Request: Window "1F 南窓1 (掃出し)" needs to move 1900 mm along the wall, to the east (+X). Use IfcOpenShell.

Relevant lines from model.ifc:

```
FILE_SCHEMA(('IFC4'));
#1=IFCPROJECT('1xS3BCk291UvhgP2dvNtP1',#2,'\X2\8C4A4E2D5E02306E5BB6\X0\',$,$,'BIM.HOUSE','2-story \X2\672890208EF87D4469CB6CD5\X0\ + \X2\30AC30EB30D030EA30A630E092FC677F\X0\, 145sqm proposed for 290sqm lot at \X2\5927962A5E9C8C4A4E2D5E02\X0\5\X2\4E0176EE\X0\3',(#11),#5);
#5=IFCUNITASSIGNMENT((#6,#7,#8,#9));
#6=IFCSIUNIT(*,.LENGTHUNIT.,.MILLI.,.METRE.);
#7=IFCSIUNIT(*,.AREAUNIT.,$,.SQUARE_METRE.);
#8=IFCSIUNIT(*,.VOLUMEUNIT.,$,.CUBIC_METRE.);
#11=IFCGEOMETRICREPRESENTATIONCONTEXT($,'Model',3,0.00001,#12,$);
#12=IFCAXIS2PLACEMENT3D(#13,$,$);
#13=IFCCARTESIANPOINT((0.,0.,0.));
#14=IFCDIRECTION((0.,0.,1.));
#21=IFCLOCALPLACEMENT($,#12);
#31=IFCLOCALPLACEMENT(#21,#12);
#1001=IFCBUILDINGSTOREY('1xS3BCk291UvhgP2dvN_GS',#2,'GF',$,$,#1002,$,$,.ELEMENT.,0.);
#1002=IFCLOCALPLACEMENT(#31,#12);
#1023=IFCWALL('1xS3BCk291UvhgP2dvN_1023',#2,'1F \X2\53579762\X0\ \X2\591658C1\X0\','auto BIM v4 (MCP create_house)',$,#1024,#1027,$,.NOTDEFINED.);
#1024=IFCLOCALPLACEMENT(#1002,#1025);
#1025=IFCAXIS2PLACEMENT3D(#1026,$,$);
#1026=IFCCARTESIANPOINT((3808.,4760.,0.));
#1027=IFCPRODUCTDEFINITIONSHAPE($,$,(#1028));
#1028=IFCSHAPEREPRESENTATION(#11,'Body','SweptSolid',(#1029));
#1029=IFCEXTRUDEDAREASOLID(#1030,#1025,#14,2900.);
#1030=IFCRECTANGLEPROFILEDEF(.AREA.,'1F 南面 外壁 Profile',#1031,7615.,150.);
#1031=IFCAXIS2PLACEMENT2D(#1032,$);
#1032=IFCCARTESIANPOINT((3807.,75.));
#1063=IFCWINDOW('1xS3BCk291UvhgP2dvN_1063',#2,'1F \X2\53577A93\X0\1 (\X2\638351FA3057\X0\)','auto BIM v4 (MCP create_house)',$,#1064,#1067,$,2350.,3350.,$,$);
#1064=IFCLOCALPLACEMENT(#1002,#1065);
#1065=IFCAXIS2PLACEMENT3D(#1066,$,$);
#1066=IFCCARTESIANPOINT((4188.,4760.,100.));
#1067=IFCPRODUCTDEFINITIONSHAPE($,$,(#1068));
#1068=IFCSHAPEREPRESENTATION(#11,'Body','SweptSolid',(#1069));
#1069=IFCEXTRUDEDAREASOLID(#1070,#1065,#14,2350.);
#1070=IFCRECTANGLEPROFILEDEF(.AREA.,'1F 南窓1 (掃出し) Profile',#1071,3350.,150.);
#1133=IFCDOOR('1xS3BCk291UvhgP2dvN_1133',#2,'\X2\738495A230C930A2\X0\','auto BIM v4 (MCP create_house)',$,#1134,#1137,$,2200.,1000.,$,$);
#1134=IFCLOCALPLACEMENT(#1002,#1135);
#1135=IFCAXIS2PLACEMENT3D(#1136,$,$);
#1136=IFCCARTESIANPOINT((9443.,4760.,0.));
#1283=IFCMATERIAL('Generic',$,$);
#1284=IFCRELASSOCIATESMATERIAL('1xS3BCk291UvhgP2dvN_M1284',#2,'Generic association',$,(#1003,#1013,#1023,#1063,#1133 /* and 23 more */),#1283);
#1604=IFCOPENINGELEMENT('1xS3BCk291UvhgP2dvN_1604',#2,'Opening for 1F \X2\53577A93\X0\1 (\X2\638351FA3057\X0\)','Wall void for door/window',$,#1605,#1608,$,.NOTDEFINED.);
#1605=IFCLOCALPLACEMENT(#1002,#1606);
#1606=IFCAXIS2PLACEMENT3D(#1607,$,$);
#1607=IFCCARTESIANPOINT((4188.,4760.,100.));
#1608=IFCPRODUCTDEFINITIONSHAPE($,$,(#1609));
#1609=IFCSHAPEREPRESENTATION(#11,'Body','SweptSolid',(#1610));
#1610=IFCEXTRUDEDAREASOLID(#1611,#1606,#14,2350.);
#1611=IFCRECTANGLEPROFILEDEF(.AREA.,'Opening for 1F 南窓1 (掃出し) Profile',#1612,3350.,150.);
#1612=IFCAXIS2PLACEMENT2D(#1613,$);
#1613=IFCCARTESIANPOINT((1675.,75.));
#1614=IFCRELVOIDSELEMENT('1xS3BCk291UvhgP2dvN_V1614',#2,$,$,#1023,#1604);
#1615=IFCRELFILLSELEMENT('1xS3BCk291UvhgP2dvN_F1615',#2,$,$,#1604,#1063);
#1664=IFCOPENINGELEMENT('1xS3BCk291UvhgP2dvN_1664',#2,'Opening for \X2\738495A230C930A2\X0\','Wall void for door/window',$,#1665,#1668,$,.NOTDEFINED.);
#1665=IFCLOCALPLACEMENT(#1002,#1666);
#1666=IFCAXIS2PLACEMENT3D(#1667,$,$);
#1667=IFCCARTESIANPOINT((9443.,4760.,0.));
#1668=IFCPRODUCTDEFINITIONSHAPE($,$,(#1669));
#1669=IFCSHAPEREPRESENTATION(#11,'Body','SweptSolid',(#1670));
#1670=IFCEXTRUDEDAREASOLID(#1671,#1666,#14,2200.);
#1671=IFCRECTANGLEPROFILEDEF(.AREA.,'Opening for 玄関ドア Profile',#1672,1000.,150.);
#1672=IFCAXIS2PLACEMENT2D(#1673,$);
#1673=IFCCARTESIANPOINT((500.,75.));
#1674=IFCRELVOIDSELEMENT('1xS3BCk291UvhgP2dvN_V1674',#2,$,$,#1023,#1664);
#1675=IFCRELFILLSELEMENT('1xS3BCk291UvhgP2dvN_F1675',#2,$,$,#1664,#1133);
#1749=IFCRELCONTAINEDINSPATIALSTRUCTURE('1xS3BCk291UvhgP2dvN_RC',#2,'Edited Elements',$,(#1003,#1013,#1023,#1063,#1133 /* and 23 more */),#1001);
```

```python
import ifcopenshell
import ifcopenshell.api.geometry
import ifcopenshell.util.placement

model = ifcopenshell.open("model.ifc")

window = model.by_id(1063)
opening = window.FillsVoids[0].RelatingOpeningElement
wall = opening.VoidsElements[0].RelatingBuildingElement

wall_matrix = ifcopenshell.util.placement.get_local_placement(wall.ObjectPlacement)
shift = wall_matrix[:3, 0] * 1900.0
before = ifcopenshell.util.placement.get_local_placement(window.ObjectPlacement)[:3, 3].copy()

# The window is not placed relative to its opening, so move both.
for product in (opening, window):
    matrix = ifcopenshell.util.placement.get_local_placement(product.ObjectPlacement)
    matrix[:3, 3] += shift
    ifcopenshell.api.geometry.edit_object_placement(model, product=product, matrix=matrix, is_si=False)

after = ifcopenshell.util.placement.get_local_placement(window.ObjectPlacement)[:3, 3]
print("window moved by", (after - before).round(3) + 0.0)

model.write("model-out.ifc")
```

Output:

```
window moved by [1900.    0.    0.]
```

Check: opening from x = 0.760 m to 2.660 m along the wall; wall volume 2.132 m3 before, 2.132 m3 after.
